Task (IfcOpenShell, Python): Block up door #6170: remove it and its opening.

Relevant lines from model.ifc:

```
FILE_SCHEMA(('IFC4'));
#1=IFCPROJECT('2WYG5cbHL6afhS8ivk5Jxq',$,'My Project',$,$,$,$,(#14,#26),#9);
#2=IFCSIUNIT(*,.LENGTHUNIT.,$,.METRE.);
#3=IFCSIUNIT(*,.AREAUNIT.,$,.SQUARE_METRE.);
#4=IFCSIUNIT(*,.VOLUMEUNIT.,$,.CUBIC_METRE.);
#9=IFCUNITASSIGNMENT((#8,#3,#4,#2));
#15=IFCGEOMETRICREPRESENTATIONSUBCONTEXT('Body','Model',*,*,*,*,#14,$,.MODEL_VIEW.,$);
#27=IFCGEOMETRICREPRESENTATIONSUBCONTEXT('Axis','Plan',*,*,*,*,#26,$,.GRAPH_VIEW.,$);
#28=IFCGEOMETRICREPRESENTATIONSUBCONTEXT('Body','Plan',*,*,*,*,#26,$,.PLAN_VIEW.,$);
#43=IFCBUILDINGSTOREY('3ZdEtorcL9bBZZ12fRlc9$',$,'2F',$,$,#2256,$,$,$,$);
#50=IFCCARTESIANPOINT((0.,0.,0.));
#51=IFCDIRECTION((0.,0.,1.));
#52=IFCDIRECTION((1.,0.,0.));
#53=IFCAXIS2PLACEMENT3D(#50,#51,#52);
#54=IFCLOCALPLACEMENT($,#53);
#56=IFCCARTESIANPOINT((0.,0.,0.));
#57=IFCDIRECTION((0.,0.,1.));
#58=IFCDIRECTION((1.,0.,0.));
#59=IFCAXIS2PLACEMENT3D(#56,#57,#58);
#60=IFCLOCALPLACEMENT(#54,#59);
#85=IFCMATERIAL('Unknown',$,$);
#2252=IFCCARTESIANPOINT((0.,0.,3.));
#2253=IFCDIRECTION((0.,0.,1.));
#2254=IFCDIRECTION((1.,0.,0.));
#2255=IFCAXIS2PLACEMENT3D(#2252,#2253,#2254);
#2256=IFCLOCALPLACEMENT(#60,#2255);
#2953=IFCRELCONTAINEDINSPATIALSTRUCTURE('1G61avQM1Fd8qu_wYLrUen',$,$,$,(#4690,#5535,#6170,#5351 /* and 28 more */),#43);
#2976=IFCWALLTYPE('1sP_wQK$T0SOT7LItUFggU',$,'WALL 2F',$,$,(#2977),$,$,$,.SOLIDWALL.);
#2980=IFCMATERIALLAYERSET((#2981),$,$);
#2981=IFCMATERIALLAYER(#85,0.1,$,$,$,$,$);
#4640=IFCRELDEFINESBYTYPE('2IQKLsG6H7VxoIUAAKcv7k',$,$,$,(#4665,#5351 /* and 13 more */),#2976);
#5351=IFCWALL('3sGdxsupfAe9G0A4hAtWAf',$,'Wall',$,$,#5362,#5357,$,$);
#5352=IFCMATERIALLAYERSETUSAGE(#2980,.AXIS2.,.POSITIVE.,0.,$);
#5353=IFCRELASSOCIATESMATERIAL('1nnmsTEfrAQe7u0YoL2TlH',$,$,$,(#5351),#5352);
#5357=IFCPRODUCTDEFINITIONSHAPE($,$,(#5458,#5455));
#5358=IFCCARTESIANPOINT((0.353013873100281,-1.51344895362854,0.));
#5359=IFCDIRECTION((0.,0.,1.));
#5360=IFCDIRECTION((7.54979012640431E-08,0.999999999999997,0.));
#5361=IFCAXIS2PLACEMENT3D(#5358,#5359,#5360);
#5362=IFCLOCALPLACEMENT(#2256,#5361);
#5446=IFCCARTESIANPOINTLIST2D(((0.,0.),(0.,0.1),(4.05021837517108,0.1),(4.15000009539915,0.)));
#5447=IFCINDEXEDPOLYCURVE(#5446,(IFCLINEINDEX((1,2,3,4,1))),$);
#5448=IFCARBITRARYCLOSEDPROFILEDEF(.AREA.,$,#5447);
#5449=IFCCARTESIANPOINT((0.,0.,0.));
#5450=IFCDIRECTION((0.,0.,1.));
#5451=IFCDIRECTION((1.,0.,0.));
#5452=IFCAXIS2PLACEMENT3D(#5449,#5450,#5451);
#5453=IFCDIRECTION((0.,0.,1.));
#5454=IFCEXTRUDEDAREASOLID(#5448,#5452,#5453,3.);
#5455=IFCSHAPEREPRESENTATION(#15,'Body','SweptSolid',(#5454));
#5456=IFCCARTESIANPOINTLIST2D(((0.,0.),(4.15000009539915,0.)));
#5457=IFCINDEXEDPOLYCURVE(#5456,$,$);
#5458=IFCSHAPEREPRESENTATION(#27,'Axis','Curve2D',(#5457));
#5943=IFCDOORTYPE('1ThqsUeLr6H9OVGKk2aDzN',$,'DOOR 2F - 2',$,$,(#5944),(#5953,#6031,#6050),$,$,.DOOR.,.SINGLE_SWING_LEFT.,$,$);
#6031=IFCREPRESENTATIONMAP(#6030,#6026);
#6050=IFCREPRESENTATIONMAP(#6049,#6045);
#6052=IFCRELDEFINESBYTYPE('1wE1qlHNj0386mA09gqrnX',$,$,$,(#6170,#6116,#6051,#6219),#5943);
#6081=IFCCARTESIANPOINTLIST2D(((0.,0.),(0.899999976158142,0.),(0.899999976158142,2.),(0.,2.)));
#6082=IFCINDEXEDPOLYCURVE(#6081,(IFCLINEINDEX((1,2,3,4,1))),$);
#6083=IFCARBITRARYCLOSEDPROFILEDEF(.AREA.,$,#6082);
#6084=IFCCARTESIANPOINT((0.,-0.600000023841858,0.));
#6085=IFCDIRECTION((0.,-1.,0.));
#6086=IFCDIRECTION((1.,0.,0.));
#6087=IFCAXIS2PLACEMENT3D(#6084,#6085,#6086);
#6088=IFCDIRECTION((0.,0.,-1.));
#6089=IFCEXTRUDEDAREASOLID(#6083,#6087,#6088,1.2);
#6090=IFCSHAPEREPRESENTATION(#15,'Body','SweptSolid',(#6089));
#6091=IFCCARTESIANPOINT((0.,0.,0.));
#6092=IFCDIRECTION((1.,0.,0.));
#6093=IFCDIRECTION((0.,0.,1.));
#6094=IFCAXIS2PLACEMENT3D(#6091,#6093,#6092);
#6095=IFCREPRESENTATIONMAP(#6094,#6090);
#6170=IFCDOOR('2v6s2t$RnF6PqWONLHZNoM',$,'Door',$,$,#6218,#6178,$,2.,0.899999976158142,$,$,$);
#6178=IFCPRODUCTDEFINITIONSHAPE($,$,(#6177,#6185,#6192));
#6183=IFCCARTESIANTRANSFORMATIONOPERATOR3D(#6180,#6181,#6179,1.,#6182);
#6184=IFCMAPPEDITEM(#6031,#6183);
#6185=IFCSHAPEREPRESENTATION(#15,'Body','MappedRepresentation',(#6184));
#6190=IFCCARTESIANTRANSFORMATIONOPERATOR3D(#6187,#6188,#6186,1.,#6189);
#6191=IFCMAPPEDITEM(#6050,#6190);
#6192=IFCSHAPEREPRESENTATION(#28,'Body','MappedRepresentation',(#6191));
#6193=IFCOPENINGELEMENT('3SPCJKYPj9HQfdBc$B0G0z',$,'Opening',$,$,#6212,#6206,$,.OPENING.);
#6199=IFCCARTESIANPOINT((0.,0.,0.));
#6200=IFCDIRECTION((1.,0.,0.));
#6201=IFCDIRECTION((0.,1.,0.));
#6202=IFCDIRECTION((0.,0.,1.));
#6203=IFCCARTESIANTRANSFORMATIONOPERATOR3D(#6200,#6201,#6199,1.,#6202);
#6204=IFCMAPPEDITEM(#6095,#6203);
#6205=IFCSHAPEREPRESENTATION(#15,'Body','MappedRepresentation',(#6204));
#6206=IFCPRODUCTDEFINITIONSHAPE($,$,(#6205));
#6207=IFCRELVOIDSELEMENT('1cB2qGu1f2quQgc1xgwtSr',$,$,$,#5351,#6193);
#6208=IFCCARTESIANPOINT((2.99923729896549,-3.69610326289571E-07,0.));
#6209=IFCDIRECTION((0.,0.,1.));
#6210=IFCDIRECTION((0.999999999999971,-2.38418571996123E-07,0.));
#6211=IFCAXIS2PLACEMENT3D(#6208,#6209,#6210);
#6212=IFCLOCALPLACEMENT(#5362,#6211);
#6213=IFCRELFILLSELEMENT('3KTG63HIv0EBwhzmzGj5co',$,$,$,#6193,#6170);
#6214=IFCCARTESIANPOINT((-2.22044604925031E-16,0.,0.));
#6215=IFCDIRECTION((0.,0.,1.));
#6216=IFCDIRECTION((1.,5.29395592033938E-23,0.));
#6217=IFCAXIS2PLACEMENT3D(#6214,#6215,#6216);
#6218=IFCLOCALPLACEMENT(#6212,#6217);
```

```python
import ifcopenshell
import ifcopenshell.api.feature
import ifcopenshell.api.root
import ifcopenshell.geom
import ifcopenshell.util.shape

model = ifcopenshell.open("model.ifc")
settings = ifcopenshell.geom.settings()


def volume(element):
    """Net volume in cubic metres, openings subtracted."""
    shape = ifcopenshell.geom.create_shape(settings, element)
    return ifcopenshell.util.shape.get_volume(shape.geometry)


door = model.by_id(6170)
opening = door.FillsVoids[0].RelatingOpeningElement
wall = opening.VoidsElements[0].RelatingBuildingElement
before = volume(wall)

ifcopenshell.api.root.remove_product(model, product=door)
ifcopenshell.api.feature.remove_feature(model, feature=opening)

after = volume(wall)

print(f"wall volume {before:.3f} -> {after:.3f} m3")

model.write("model_rev.ifc")
```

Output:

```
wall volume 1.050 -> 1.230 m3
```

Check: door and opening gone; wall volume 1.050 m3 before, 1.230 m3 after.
